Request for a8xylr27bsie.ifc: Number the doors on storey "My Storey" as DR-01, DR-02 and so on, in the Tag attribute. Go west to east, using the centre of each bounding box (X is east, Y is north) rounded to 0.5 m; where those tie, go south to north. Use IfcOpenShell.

First a look at what the model holds.

```python
import ifcopenshell
import ifcopenshell.util.element
import ifcopenshell.util.placement

model = ifcopenshell.open("a8xylr27bsie.ifc")
print(model.schema)
storey = next(s for s in model.by_type("IfcBuildingStorey") if s.Name == "My Storey")
doors = [e for e in ifcopenshell.util.element.get_decomposition(storey) if e.is_a("IfcDoor")]
for e in sorted(doors, key=lambda e: e.id()):
    origin = ifcopenshell.util.placement.get_local_placement(e.ObjectPlacement)[:3, 3]
    print(e.id(), e.Tag, e.Name, origin.round(2) + 0.0, sep=" | ")
```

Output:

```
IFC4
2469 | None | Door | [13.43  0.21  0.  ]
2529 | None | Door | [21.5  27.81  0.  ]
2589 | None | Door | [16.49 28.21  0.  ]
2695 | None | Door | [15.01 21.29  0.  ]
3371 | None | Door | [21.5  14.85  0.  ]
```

```python
import ifcopenshell
import ifcopenshell.geom
import ifcopenshell.util.element
import ifcopenshell.util.shape

model = ifcopenshell.open("a8xylr27bsie.ifc")
settings = ifcopenshell.geom.settings()
settings.set("use-world-coords", True)


def centre(element):
    shape = ifcopenshell.geom.create_shape(settings, element)
    return ifcopenshell.util.shape.get_bbox_centroid(shape.geometry)


storey = next(s for s in model.by_type("IfcBuildingStorey") if s.Name == "My Storey")
doors = [e for e in ifcopenshell.util.element.get_decomposition(storey) if e.is_a("IfcDoor")]

# Insertion points can sit at a corner or the storey origin, so sort by the geometry (in metres).
centres = {e: centre(e) for e in doors}
doors.sort(key=lambda e: (round(centres[e][0] / 0.5), centres[e][1]))

for i, e in enumerate(doors, start=1):
    number = f"DR-{i:02d}"
    e.Tag = number
    print(e.id(), number)

model.write("a8xylr27bsie_rev.ifc")
```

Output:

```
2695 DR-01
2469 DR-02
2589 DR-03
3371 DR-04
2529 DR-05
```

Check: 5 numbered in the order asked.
